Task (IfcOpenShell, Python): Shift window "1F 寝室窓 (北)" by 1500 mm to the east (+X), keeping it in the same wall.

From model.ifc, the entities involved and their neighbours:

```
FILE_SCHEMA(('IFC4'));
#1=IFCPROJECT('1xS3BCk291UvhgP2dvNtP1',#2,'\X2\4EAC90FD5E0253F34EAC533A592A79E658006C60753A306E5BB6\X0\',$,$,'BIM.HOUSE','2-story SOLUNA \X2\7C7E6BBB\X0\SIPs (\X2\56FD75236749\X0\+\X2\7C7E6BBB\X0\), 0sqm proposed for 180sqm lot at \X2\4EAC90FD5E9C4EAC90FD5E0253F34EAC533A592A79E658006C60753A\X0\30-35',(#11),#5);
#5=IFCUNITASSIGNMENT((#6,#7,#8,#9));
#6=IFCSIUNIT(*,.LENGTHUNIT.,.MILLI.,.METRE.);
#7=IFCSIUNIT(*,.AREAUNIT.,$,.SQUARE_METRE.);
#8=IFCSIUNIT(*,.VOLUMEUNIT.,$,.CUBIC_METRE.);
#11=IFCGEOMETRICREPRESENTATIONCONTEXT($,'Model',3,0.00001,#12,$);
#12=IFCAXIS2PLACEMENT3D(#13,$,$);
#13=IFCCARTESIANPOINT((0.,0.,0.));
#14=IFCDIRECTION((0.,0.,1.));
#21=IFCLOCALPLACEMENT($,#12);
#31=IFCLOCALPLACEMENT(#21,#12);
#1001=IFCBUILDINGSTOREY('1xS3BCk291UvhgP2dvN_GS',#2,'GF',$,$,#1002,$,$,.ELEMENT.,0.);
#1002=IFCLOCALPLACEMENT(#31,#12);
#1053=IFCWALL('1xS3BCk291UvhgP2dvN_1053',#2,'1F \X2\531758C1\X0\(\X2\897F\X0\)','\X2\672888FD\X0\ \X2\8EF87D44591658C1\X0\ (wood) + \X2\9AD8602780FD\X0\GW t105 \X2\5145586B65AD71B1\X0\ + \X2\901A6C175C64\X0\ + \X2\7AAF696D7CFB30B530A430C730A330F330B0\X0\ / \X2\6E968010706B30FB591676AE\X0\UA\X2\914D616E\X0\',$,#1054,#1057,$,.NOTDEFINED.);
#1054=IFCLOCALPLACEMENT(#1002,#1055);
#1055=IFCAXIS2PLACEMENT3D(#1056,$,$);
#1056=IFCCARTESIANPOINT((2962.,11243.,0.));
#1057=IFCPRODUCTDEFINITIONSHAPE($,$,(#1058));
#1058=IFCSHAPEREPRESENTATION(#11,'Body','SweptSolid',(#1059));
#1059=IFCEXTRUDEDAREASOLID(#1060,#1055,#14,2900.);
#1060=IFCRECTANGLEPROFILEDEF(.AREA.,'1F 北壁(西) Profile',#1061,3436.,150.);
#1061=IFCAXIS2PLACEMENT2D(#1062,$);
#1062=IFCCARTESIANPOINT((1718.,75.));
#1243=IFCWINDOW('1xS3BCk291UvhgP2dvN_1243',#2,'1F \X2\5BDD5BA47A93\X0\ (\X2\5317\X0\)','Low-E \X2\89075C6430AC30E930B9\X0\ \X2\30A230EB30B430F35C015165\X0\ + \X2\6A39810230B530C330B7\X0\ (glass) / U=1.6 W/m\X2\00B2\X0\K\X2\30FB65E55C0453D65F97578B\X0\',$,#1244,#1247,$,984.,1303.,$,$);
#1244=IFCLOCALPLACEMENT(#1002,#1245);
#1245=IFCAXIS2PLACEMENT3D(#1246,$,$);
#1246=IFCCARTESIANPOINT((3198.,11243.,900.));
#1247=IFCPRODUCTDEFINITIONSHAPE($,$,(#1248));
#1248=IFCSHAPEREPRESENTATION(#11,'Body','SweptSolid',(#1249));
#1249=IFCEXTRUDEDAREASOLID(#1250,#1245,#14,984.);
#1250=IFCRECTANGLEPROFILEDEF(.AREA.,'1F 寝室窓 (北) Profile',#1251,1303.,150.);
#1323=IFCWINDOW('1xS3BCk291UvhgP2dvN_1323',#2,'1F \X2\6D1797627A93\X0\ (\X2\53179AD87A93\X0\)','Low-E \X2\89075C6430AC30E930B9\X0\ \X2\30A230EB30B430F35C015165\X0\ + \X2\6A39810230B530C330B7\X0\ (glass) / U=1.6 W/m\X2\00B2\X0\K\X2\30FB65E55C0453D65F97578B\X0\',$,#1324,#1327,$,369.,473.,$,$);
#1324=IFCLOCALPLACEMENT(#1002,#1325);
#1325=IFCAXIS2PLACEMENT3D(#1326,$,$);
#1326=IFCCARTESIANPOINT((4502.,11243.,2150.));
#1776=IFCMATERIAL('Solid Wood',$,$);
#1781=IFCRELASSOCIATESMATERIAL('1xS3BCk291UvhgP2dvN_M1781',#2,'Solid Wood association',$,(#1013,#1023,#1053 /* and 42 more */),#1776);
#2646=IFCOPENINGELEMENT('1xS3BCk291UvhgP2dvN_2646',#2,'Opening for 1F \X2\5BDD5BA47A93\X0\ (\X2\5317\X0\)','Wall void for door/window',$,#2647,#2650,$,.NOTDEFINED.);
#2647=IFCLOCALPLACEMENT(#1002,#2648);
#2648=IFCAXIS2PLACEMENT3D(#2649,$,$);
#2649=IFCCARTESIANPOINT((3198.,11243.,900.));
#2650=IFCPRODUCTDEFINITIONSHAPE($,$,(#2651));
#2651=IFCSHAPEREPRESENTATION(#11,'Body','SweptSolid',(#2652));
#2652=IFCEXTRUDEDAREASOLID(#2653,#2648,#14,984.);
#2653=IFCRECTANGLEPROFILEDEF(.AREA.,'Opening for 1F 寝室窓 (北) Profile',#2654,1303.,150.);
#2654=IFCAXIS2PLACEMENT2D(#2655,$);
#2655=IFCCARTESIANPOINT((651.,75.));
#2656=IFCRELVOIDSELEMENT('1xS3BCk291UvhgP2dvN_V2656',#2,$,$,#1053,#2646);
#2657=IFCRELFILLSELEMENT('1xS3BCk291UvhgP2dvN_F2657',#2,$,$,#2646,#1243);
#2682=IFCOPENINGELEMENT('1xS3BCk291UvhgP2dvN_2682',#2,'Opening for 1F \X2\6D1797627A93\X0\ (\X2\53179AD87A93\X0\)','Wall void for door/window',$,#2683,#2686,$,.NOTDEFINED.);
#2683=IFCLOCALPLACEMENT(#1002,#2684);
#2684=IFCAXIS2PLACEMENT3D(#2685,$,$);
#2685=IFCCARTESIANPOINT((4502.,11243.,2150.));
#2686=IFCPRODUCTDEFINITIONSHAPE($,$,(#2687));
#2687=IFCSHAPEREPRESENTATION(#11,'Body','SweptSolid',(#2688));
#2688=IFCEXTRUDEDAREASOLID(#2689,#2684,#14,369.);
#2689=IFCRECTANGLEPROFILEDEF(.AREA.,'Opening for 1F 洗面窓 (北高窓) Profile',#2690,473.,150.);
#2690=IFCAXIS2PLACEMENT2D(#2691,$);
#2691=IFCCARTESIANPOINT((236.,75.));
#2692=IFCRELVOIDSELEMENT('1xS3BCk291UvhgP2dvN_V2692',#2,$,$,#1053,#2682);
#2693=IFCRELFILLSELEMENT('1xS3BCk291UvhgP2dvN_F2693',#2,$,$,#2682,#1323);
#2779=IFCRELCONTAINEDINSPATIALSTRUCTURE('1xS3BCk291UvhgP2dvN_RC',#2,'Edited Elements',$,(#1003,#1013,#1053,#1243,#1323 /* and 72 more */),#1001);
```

```python
import ifcopenshell
import ifcopenshell.api.geometry
import ifcopenshell.util.placement

model = ifcopenshell.open("model.ifc")

window = model.by_guid("1xS3BCk291UvhgP2dvN_1243")
opening = window.FillsVoids[0].RelatingOpeningElement
wall = opening.VoidsElements[0].RelatingBuildingElement

wall_matrix = ifcopenshell.util.placement.get_local_placement(wall.ObjectPlacement)
shift = wall_matrix[:3, 0] * 1500.0
before = ifcopenshell.util.placement.get_local_placement(window.ObjectPlacement)[:3, 3].copy()

# The window is not placed relative to its opening, so move both.
for product in (opening, window):
    matrix = ifcopenshell.util.placement.get_local_placement(product.ObjectPlacement)
    matrix[:3, 3] += shift
    ifcopenshell.api.geometry.edit_object_placement(model, product=product, matrix=matrix, is_si=False)

after = ifcopenshell.util.placement.get_local_placement(window.ObjectPlacement)[:3, 3]
print("window moved by", (after - before).round(3) + 0.0)

model.write("model-out.ifc")
```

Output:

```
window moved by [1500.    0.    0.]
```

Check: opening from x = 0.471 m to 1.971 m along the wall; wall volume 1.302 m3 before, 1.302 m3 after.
